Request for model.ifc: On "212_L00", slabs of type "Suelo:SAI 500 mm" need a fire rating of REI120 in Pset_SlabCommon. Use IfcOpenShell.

First a look at what the model holds.

```python
import ifcopenshell
import ifcopenshell.util.element

model = ifcopenshell.open("model.ifc")
print(model.schema)
storey = next(s for s in model.by_type("IfcBuildingStorey") if s.Name == "212_L00")
slabs = [e for e in ifcopenshell.util.element.get_decomposition(storey) if e.is_a("IfcSlab")]
seen = {}
for e in slabs:
    element_type = ifcopenshell.util.element.get_type(e)
    key = (element_type.Name if element_type != e and element_type else None, ifcopenshell.util.element.get_pset(e, "Pset_SlabCommon", "FireRating"))
    seen[key] = seen.get(key, 0) + 1
for (name, value), count in sorted(seen.items(), key=str):
    print(count, "x", name, "|", value)
```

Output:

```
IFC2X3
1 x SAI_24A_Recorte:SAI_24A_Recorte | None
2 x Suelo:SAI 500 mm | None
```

```python
import ifcopenshell
import ifcopenshell.api.pset
import ifcopenshell.util.element

model = ifcopenshell.open("model.ifc")

storey = next(s for s in model.by_type("IfcBuildingStorey") if s.Name == "212_L00")
slabs = [e for e in ifcopenshell.util.element.get_decomposition(storey) if e.is_a("IfcSlab")]

count = 0
for e in slabs:
    element_type = ifcopenshell.util.element.get_type(e)
    if element_type in (None, e) or element_type.Name != "Suelo:SAI 500 mm":
        continue
    # add_pset returns the element's existing set when there is one.
    pset = ifcopenshell.api.pset.add_pset(model, product=e, name="Pset_SlabCommon")
    ifcopenshell.api.pset.edit_pset(model, pset=pset, properties={"FireRating": "REI120"})
    count += 1

print(count, "slabs updated")

model.write("model_updated.ifc")
```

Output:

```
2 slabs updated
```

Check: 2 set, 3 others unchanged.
